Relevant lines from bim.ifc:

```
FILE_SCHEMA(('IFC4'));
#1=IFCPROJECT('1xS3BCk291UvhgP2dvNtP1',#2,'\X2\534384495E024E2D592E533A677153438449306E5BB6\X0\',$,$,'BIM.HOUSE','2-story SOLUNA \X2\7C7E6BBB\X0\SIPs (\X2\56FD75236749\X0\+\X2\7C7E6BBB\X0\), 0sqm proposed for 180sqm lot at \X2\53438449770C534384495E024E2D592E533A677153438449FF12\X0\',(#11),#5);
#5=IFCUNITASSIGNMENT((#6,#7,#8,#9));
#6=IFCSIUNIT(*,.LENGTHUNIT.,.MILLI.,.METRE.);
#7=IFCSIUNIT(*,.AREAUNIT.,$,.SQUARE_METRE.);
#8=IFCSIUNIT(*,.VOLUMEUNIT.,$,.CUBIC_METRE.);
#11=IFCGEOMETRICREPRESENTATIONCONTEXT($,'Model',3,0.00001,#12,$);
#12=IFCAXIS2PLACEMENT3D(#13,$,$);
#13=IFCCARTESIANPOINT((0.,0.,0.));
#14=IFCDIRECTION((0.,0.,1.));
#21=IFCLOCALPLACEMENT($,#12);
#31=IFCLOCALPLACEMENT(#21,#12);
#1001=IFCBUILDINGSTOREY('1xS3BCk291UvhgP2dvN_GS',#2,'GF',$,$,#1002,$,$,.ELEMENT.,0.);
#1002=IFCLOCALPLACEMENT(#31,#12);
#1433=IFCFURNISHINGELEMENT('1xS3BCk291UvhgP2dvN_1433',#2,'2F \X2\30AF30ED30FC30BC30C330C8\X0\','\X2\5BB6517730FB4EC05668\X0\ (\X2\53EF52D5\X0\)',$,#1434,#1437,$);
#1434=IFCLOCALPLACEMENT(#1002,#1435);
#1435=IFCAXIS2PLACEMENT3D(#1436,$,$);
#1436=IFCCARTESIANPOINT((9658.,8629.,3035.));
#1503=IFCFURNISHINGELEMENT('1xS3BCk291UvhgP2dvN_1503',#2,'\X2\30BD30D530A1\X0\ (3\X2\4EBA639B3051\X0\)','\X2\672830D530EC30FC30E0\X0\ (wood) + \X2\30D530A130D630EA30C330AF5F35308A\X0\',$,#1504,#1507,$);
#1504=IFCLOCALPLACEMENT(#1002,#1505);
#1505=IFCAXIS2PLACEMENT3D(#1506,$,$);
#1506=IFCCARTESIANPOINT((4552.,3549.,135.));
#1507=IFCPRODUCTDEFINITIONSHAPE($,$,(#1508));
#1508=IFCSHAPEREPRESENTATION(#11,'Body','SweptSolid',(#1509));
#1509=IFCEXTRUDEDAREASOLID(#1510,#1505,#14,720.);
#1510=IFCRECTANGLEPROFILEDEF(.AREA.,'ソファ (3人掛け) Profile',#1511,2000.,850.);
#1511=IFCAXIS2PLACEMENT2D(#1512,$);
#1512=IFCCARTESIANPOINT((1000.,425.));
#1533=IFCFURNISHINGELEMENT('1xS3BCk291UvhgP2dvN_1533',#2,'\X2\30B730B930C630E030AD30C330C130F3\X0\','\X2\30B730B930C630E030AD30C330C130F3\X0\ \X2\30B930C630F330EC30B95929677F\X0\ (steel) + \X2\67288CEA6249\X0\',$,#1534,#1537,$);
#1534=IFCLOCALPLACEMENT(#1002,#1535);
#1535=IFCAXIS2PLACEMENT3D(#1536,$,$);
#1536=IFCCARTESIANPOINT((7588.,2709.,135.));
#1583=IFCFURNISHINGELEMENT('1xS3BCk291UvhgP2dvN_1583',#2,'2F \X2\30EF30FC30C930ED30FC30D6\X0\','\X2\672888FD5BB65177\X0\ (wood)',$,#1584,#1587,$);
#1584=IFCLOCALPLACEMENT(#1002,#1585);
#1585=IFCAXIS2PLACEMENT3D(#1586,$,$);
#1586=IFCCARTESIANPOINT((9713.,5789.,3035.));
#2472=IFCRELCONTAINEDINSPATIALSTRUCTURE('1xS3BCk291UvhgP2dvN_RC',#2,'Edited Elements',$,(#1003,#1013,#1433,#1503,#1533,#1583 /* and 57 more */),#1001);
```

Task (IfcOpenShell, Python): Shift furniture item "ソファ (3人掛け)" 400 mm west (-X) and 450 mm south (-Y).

```python
import ifcopenshell
import ifcopenshell.api.geometry
import ifcopenshell.util.placement

model = ifcopenshell.open("bim.ifc")

item = model.by_guid("1xS3BCk291UvhgP2dvN_1503")
matrix = ifcopenshell.util.placement.get_local_placement(item.ObjectPlacement)
matrix[0, 3] -= 400.0
matrix[1, 3] -= 450.0
ifcopenshell.api.geometry.edit_object_placement(model, product=item, matrix=matrix, is_si=False)

print(ifcopenshell.util.placement.get_local_placement(item.ObjectPlacement).round(3) + 0.0)

model.write("bim_edited.ifc")
```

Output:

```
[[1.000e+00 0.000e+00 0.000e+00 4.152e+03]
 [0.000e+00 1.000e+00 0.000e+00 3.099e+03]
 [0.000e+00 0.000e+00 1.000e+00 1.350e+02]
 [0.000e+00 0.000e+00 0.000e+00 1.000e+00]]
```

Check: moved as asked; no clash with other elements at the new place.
